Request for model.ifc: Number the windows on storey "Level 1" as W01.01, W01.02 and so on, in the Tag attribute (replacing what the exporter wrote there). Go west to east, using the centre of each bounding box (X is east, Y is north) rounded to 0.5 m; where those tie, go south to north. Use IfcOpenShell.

First a look at what the model holds.

```python
import ifcopenshell
import ifcopenshell.util.element
import ifcopenshell.util.placement

model = ifcopenshell.open("model.ifc")
print(model.schema)
storey = next(s for s in model.by_type("IfcBuildingStorey") if s.Name == "Level 1")
windows = [e for e in ifcopenshell.util.element.get_decomposition(storey) if e.is_a("IfcWindow")]
for e in sorted(windows, key=lambda e: e.id()):
    origin = ifcopenshell.util.placement.get_local_placement(e.ObjectPlacement)[:3, 3]
    print(e.id(), e.Tag, e.Name, origin.round(2) + 0.0, sep=" | ")
```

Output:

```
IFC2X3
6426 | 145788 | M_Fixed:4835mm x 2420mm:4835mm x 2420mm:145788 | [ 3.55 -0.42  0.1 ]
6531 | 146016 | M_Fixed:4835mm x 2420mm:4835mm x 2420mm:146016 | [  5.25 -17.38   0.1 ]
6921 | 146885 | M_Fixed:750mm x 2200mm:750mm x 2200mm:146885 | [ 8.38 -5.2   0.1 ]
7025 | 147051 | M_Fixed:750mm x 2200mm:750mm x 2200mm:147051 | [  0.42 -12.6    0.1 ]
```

```python
import ifcopenshell
import ifcopenshell.geom
import ifcopenshell.util.element
import ifcopenshell.util.shape

model = ifcopenshell.open("model.ifc")
settings = ifcopenshell.geom.settings()
settings.set("use-world-coords", True)


def centre(element):
    shape = ifcopenshell.geom.create_shape(settings, element)
    return ifcopenshell.util.shape.get_bbox_centroid(shape.geometry)


storey = next(s for s in model.by_type("IfcBuildingStorey") if s.Name == "Level 1")
windows = [e for e in ifcopenshell.util.element.get_decomposition(storey) if e.is_a("IfcWindow")]

# Insertion points can sit at a corner or the storey origin, so sort by the geometry (in metres).
centres = {e: centre(e) for e in windows}
windows.sort(key=lambda e: (round(centres[e][0] / 0.5), centres[e][1]))

for i, e in enumerate(windows, start=1):
    number = f"W01.{i:02d}"
    e.Tag = number
    print(e.id(), number)

model.write("model-out.ifc")
```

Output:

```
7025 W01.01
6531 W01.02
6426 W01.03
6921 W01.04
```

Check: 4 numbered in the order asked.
